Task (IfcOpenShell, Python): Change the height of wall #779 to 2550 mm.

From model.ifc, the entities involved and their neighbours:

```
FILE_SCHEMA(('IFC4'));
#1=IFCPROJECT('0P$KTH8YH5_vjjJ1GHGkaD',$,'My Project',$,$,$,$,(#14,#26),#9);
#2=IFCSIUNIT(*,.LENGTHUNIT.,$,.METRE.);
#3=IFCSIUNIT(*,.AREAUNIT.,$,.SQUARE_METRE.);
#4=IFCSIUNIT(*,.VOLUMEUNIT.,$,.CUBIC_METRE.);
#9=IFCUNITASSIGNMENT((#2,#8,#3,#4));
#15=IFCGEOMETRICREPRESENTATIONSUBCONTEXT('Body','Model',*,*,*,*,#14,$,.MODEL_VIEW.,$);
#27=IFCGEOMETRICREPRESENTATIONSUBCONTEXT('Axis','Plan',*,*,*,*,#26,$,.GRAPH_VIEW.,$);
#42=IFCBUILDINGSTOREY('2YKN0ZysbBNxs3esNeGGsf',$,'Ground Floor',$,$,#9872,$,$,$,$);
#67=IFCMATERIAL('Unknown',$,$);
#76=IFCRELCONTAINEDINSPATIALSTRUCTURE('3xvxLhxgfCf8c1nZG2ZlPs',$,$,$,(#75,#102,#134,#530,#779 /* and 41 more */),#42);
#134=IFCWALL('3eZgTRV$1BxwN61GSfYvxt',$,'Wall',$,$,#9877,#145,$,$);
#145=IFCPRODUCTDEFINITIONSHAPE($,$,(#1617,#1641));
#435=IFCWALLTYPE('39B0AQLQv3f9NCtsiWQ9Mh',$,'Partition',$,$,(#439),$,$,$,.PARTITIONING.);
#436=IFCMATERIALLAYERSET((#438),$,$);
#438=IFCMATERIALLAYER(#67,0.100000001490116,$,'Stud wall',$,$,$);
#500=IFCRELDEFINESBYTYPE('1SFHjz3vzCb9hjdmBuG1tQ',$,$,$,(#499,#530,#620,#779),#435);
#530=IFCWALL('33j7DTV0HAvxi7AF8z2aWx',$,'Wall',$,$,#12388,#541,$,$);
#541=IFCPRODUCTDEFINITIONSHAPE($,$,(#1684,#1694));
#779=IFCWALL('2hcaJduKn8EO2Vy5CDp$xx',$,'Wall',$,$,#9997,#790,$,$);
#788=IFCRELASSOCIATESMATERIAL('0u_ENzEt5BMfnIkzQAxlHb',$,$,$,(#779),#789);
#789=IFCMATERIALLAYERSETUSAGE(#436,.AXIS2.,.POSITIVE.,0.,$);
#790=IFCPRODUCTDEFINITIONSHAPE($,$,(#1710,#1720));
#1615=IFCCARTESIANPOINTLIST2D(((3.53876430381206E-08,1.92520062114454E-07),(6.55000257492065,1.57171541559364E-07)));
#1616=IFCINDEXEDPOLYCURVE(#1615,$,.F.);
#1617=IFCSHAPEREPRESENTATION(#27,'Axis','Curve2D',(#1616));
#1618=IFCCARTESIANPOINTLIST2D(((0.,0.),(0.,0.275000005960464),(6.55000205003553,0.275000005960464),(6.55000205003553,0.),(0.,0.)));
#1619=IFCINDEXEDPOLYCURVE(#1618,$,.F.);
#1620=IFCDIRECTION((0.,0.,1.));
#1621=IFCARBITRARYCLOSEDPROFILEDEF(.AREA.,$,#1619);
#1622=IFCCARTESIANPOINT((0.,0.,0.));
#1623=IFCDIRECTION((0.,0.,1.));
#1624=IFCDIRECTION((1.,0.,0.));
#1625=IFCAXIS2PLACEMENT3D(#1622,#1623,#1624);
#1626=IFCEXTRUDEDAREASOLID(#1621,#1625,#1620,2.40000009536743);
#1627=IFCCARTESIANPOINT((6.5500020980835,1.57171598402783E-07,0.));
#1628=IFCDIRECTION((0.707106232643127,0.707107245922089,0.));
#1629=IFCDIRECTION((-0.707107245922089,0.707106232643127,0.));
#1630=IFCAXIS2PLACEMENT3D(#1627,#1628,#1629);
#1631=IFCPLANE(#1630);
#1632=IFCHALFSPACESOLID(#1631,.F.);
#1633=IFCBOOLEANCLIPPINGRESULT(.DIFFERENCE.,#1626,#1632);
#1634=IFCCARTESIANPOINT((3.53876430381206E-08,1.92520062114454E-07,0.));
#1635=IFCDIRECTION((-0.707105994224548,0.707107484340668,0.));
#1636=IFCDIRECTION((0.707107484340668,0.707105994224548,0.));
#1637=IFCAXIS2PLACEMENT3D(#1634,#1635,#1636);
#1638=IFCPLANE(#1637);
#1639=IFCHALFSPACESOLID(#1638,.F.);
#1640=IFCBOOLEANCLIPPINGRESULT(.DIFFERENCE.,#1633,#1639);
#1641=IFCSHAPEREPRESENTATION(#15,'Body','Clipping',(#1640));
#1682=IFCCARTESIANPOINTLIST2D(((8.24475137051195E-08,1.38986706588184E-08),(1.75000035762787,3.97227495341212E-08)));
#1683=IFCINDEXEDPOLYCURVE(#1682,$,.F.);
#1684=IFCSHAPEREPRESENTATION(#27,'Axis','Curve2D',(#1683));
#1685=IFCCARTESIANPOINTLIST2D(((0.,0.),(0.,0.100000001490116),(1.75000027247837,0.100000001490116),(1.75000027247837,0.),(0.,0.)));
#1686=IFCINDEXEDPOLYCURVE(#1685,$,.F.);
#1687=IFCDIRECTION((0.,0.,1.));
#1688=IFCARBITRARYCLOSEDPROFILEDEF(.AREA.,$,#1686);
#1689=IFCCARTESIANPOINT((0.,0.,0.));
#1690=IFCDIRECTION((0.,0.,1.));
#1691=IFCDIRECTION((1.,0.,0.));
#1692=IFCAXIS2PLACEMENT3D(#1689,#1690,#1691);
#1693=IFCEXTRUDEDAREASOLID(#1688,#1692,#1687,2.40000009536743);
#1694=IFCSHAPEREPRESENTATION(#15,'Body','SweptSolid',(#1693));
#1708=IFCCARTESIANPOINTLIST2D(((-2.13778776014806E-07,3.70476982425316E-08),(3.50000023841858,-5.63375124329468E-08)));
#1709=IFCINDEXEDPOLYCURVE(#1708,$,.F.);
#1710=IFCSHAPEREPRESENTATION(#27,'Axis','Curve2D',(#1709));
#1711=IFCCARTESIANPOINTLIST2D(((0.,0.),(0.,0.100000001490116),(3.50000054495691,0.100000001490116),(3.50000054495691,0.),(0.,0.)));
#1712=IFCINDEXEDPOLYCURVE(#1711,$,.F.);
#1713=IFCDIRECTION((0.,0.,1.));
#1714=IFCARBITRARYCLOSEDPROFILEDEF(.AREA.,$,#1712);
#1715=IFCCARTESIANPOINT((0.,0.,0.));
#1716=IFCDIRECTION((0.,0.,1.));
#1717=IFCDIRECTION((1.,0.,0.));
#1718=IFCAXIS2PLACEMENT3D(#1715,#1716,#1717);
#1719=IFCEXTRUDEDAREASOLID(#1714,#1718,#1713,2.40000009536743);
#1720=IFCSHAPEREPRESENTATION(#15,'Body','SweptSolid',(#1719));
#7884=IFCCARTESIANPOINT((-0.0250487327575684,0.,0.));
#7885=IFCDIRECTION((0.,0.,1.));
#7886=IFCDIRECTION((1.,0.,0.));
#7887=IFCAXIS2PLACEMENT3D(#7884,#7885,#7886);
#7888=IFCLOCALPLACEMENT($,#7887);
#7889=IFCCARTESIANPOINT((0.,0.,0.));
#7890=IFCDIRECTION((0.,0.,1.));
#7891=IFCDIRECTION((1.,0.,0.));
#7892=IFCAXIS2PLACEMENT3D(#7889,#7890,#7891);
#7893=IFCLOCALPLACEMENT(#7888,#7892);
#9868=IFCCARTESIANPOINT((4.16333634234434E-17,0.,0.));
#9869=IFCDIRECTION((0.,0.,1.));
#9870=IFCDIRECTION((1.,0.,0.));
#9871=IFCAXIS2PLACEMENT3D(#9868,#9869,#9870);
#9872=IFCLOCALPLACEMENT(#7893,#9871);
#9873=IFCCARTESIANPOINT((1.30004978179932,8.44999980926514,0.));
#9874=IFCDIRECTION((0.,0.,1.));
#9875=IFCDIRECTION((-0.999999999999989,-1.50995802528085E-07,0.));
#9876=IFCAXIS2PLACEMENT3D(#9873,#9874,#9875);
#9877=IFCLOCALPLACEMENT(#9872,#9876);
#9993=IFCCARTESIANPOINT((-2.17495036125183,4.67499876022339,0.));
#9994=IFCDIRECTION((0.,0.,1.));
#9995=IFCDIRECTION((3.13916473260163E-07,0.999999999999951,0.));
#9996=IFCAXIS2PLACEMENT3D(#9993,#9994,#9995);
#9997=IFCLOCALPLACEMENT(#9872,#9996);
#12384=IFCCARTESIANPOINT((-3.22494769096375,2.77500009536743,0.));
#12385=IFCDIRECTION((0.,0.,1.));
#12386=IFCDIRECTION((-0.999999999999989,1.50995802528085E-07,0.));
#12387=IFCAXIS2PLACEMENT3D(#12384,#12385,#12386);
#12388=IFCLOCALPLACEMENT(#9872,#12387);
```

```python
import ifcopenshell
import ifcopenshell.geom
import ifcopenshell.util.representation
import ifcopenshell.util.shape

model = ifcopenshell.open("model.ifc")
settings = ifcopenshell.geom.settings()


def volume(element):
    """Net volume in cubic metres, openings subtracted."""
    shape = ifcopenshell.geom.create_shape(settings, element)
    return ifcopenshell.util.shape.get_volume(shape.geometry)


wall = model.by_guid("2hcaJduKn8EO2Vy5CDp$xx")
before = volume(wall)

body = ifcopenshell.util.representation.get_representation(wall, "Model", "Body")
solid = body.Items[0]
old_height = solid.Depth
solid.Depth = 2.55
after = volume(wall)

print(f"height {old_height:g} -> {solid.Depth:g}, volume {before:.3f} -> {after:.3f} m3")

model.write("model_edited.ifc")
```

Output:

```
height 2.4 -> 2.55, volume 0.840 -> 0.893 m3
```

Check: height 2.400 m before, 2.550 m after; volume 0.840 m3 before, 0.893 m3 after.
